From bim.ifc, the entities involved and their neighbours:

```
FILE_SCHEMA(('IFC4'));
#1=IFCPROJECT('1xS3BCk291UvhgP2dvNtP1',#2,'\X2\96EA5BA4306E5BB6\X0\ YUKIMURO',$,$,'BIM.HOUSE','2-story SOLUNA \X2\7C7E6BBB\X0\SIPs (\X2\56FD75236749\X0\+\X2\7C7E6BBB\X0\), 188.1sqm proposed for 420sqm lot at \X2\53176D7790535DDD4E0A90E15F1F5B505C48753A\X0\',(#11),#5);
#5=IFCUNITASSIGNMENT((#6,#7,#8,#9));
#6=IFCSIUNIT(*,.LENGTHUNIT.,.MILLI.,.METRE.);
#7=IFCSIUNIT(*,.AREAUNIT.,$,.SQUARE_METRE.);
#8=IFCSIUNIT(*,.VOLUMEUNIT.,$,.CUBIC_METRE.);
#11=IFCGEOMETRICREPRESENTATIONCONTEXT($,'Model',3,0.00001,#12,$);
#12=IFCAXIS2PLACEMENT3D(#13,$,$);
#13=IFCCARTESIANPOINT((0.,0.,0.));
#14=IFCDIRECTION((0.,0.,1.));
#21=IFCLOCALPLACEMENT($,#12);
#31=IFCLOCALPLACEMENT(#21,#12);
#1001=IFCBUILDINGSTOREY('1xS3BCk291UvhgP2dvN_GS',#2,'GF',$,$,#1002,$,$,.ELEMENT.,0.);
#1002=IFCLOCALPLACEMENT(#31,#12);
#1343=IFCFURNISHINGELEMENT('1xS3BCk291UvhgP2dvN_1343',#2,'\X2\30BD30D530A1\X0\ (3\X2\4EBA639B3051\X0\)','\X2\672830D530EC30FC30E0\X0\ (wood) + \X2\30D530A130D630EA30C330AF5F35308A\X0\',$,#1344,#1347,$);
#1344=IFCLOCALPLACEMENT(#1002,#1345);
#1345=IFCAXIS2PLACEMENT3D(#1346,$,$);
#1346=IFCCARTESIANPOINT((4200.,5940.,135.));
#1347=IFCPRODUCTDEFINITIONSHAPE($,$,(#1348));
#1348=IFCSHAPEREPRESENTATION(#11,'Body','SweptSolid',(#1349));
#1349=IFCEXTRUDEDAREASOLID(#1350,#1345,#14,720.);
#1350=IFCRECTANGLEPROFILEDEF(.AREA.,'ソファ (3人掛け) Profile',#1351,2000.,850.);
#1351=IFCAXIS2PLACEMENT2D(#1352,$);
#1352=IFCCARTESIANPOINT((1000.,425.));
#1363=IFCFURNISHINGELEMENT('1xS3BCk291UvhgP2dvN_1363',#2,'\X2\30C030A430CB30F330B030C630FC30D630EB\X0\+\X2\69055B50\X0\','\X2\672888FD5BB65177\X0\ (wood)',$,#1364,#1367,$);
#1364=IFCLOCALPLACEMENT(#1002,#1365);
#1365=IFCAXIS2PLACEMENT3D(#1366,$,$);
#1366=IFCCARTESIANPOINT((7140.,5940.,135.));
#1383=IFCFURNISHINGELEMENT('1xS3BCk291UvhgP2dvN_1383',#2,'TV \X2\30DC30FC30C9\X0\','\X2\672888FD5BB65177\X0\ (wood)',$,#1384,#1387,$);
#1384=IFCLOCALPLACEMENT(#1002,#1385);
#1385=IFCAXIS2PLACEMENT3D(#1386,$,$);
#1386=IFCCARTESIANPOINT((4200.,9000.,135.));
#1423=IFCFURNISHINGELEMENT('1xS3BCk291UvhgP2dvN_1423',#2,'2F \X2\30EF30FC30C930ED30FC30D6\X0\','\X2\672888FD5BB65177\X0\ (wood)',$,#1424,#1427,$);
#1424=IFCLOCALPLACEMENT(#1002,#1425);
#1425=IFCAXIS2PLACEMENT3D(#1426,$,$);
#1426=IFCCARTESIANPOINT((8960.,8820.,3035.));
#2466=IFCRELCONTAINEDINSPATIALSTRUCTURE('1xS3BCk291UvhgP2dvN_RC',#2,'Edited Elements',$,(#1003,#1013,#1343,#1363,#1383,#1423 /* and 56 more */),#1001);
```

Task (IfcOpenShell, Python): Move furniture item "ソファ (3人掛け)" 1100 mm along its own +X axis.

```python
import ifcopenshell
import ifcopenshell.api.geometry
import ifcopenshell.util.placement

model = ifcopenshell.open("bim.ifc")

item = model.by_guid("1xS3BCk291UvhgP2dvN_1343")
matrix = ifcopenshell.util.placement.get_local_placement(item.ObjectPlacement)
matrix[:3, 3] += matrix[:3, 0] * 1100.0
ifcopenshell.api.geometry.edit_object_placement(model, product=item, matrix=matrix, is_si=False)

print(ifcopenshell.util.placement.get_local_placement(item.ObjectPlacement).round(3) + 0.0)

model.write("bim_edited.ifc")
```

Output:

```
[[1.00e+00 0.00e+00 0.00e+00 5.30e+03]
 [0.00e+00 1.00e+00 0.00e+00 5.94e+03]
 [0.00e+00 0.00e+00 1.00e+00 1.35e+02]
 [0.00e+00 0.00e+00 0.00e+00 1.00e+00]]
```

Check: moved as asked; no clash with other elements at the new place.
